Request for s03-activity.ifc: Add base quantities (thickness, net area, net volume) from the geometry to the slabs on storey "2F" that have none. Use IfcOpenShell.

First a look at what the model holds.

```python
import ifcopenshell
import ifcopenshell.util.element
import ifcopenshell.util.unit

model = ifcopenshell.open("s03-activity.ifc")
print(model.schema)
for unit_type in ("LENGTHUNIT", "AREAUNIT", "VOLUMEUNIT"):
    print(unit_type, ifcopenshell.util.unit.calculate_unit_scale(model, unit_type))
storey = next(s for s in model.by_type("IfcBuildingStorey") if s.Name == "2F")
slabs = [e for e in ifcopenshell.util.element.get_decomposition(storey) if e.is_a("IfcSlab")]
for e in sorted(slabs, key=lambda e: e.id()):
    print(e.id(), e.is_a(), e.Name, list(ifcopenshell.util.element.get_psets(e, qtos_only=True)), sep=" | ")
```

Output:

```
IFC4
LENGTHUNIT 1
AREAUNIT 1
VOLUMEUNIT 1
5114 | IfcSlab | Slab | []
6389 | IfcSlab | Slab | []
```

```python
import ifcopenshell
import ifcopenshell.api.pset
import ifcopenshell.geom
import ifcopenshell.util.element
import ifcopenshell.util.shape
import ifcopenshell.util.unit

model = ifcopenshell.open("s03-activity.ifc")
unit_scale = ifcopenshell.util.unit.calculate_unit_scale(model)
area_scale = ifcopenshell.util.unit.calculate_unit_scale(model, "AREAUNIT")
volume_scale = ifcopenshell.util.unit.calculate_unit_scale(model, "VOLUMEUNIT")
settings = ifcopenshell.geom.settings()

storey = next(s for s in model.by_type("IfcBuildingStorey") if s.Name == "2F")
slabs = [e for e in ifcopenshell.util.element.get_decomposition(storey) if e.is_a("IfcSlab")]

for e in sorted(slabs, key=lambda e: e.id()):
    if ifcopenshell.util.element.get_psets(e, qtos_only=True, should_inherit=False):
        continue
    # Geometry comes back in metres, in the element's own axes.
    shape = ifcopenshell.geom.create_shape(settings, e)
    values = {
        "Width": ifcopenshell.util.shape.get_z(shape.geometry) / unit_scale,
        "NetArea": ifcopenshell.util.shape.get_footprint_area(shape.geometry) / area_scale,
        "NetVolume": ifcopenshell.util.shape.get_volume(shape.geometry) / volume_scale,
    }
    qto = ifcopenshell.api.pset.add_qto(model, product=e, name="Qto_SlabBaseQuantities")
    ifcopenshell.api.pset.edit_qto(model, qto=qto, properties=values)
    print(e.id(), {k: round(v, 3) for k, v in values.items()})

model.write("s03-activity_v2.ifc")
```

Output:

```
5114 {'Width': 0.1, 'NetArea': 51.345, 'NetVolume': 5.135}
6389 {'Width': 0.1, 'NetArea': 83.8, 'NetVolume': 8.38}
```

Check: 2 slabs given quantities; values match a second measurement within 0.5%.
